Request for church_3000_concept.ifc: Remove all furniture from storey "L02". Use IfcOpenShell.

First a look at what the model holds.

```python
import ifcopenshell
import ifcopenshell.util.element

model = ifcopenshell.open("church_3000_concept.ifc")
print(model.schema)
storey = next(s for s in model.by_type("IfcBuildingStorey") if s.Name == "L02")
furniture = [e for e in ifcopenshell.util.element.get_decomposition(storey) if e.is_a("IfcFurnishingElement")]
seen = {}
for e in furniture:
    element_type = ifcopenshell.util.element.get_type(e)
    name = element_type.Name if element_type not in (None, e) else None
    seen[name] = seen.get(name, 0) + 1
for name, count in sorted(seen.items(), key=str):
    print(count, "x", name)
```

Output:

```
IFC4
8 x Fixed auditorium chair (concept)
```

```python
import ifcopenshell
import ifcopenshell.api.root
import ifcopenshell.util.element

model = ifcopenshell.open("church_3000_concept.ifc")

storey = next(s for s in model.by_type("IfcBuildingStorey") if s.Name == "L02")
furniture = [e for e in ifcopenshell.util.element.get_decomposition(storey) if e.is_a("IfcFurnishingElement")]

for e in furniture:
    ifcopenshell.api.root.remove_product(model, product=e)
print(len(furniture), "removed")

model.write("church_3000_concept_rev.ifc")
```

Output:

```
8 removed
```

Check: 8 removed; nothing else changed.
